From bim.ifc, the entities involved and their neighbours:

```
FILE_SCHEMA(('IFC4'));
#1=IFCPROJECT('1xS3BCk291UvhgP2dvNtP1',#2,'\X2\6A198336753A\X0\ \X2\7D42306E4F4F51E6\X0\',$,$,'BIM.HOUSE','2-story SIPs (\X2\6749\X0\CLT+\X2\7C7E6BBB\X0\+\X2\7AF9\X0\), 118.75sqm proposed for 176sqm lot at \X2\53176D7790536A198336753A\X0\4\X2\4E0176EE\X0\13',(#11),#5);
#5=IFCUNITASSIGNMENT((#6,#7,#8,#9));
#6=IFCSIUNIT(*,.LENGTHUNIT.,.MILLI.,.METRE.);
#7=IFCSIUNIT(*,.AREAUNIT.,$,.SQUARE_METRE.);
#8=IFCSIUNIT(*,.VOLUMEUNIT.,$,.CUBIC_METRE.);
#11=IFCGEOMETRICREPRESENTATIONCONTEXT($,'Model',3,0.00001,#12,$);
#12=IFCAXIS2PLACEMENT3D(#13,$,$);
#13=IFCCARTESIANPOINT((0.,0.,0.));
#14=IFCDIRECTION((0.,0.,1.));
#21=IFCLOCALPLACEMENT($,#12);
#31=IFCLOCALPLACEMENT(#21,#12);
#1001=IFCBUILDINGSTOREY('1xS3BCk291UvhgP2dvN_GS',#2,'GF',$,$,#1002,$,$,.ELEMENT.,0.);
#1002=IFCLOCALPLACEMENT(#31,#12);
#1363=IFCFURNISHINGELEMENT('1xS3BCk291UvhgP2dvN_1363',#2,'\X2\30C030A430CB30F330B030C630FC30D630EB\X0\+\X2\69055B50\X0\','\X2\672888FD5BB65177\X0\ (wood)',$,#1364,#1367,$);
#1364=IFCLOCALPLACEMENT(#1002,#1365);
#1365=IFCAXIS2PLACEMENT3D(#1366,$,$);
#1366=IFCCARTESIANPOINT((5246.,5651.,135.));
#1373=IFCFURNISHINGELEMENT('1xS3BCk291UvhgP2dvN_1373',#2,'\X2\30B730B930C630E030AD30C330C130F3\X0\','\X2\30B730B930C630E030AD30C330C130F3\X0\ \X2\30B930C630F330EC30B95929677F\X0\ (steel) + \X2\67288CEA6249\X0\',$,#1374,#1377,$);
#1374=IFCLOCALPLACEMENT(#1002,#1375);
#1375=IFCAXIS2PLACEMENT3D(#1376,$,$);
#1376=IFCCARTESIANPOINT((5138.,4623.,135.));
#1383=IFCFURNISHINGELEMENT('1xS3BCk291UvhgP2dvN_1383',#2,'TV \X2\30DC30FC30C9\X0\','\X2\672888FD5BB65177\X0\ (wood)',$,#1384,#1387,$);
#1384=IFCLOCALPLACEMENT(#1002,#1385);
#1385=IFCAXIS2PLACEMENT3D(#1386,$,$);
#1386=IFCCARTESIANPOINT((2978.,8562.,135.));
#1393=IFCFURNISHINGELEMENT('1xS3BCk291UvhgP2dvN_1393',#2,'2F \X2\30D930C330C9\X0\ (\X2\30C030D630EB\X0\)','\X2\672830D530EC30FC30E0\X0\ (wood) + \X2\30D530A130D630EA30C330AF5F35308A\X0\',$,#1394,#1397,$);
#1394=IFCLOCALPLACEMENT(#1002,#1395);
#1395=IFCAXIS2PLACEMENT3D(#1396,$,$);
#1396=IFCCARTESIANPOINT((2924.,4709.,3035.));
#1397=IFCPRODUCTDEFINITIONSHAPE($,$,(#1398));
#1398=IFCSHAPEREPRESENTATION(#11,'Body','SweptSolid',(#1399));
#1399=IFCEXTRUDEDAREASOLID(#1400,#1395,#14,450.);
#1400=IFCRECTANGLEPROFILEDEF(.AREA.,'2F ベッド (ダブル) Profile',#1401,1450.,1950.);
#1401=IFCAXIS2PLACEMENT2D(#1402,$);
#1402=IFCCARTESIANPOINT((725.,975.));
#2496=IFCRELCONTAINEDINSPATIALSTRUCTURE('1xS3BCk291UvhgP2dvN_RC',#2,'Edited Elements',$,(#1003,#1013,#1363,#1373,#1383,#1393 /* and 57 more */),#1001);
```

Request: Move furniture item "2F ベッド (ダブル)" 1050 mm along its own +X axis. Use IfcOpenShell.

```python
import ifcopenshell
import ifcopenshell.api.geometry
import ifcopenshell.util.placement
import ifcopenshell.util.unit

model = ifcopenshell.open("bim.ifc")
unit_scale = ifcopenshell.util.unit.calculate_unit_scale(model)

item = model.by_guid("1xS3BCk291UvhgP2dvN_1393")
matrix = ifcopenshell.util.placement.get_local_placement(item.ObjectPlacement)
matrix[:3, 3] += matrix[:3, 0] * 1.05 / unit_scale
ifcopenshell.api.geometry.edit_object_placement(model, product=item, matrix=matrix, is_si=False)

print(ifcopenshell.util.placement.get_local_placement(item.ObjectPlacement).round(3) + 0.0)

model.write("bim_v2.ifc")
```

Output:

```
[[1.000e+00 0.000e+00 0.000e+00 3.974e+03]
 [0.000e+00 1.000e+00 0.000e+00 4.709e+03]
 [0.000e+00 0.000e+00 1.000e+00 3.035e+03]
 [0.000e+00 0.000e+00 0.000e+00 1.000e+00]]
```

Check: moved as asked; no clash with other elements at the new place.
